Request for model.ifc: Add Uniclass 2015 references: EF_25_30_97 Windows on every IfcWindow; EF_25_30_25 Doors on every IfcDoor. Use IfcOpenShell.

First a look at what the model holds.

```python
import ifcopenshell

model = ifcopenshell.open("model.ifc")
print(model.schema)
print("classifications:", [c.Name for c in model.by_type("IfcClassification")])
for ifc_class in ("IfcDoor", "IfcRoof", "IfcStair", "IfcWall", "IfcWindow"):
    print(ifc_class, len(model.by_type(ifc_class)))
```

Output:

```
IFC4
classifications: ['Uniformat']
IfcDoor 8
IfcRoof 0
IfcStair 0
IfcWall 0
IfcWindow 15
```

```python
import ifcopenshell
import ifcopenshell.api.classification

model = ifcopenshell.open("model.ifc")

system = ifcopenshell.api.classification.add_classification(model, classification="Uniclass 2015")

codes = {
    "IfcWindow": ("EF_25_30_97", "Windows"),
    "IfcDoor": ("EF_25_30_25", "Doors"),
}
for ifc_class, (code, name) in codes.items():
    products = model.by_type(ifc_class)
    ifcopenshell.api.classification.add_reference(
        model, products=products, classification=system, identification=code, name=name
    )
    print(code, len(products))

model.write("model_v2.ifc")
```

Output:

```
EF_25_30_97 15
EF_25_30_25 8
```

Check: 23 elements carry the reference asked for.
